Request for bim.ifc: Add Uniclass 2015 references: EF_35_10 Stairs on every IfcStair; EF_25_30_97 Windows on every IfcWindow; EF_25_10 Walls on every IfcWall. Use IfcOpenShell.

First a look at what the model holds.

```python
import ifcopenshell

model = ifcopenshell.open("bim.ifc")
print(model.schema)
print("classifications:", [c.Name for c in model.by_type("IfcClassification")])
for ifc_class in ("IfcDoor", "IfcRoof", "IfcStair", "IfcWall", "IfcWindow"):
    print(ifc_class, len(model.by_type(ifc_class)))
```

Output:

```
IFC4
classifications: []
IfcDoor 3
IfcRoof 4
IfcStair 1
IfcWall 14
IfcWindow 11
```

```python
import ifcopenshell
import ifcopenshell.api.classification

model = ifcopenshell.open("bim.ifc")

system = ifcopenshell.api.classification.add_classification(model, classification="Uniclass 2015")

codes = {
    "IfcStair": ("EF_35_10", "Stairs"),
    "IfcWindow": ("EF_25_30_97", "Windows"),
    "IfcWall": ("EF_25_10", "Walls"),
}
for ifc_class, (code, name) in codes.items():
    products = model.by_type(ifc_class)
    ifcopenshell.api.classification.add_reference(
        model, products=products, classification=system, identification=code, name=name
    )
    print(code, len(products))

model.write("bim_edited.ifc")
```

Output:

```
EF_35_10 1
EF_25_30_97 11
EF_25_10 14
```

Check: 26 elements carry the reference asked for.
